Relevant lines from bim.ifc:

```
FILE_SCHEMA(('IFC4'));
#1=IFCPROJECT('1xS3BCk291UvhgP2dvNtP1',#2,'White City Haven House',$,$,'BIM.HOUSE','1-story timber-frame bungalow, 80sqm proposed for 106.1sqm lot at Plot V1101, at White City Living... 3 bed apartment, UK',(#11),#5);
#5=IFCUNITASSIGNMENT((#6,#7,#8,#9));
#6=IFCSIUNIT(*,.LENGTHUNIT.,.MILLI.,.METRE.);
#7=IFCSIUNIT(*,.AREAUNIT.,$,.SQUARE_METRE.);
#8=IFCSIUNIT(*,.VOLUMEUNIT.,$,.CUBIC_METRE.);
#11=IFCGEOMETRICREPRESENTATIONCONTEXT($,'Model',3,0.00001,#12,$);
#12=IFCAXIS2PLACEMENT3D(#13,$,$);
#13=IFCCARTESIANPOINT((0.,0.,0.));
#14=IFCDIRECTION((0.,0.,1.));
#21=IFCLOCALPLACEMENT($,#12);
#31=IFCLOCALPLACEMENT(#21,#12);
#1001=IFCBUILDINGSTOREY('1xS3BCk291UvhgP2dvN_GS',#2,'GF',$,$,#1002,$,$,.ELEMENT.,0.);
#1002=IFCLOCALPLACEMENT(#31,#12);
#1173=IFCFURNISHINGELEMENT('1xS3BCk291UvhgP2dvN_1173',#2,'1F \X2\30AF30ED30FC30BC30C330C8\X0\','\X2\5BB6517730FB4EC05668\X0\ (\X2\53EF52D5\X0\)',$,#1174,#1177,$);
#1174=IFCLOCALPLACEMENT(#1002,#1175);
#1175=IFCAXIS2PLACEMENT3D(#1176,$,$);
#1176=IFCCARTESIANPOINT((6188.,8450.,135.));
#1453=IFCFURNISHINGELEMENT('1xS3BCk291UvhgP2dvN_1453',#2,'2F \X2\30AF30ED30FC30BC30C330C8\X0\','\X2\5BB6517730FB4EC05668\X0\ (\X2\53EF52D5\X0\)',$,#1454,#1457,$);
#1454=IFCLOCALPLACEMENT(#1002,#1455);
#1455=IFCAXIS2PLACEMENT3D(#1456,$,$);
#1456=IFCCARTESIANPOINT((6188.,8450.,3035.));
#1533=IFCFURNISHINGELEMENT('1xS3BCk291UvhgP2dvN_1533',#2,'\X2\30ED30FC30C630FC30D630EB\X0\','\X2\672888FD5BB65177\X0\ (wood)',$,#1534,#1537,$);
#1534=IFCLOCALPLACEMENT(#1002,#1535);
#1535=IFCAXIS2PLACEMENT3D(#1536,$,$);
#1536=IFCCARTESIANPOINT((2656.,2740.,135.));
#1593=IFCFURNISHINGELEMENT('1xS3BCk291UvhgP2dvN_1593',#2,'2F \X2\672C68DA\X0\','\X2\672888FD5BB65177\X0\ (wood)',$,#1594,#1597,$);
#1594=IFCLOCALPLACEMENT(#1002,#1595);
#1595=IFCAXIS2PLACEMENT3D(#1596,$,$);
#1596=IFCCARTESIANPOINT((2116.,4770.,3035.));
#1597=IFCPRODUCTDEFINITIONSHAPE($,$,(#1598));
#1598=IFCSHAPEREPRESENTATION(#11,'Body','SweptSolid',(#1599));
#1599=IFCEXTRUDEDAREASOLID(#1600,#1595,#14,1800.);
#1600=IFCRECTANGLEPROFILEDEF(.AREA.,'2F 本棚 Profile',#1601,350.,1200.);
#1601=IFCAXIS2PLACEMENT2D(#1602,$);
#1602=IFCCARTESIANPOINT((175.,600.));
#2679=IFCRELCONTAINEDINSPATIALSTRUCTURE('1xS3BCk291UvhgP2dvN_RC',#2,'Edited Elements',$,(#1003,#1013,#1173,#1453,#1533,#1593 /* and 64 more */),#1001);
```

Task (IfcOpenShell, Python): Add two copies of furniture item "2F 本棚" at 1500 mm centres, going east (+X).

```python
import numpy as np
import ifcopenshell
import ifcopenshell.api.geometry
import ifcopenshell.api.root
import ifcopenshell.util.element
import ifcopenshell.util.placement
import ifcopenshell.util.unit

model = ifcopenshell.open("bim.ifc")
unit_scale = ifcopenshell.util.unit.calculate_unit_scale(model)


def reuse_history(source, copy):
    """copy_class also copies each property set's owner history, people and application; keep the originals."""
    for rel in copy.IsDefinedBy:
        if rel.is_a("IfcRelDefinesByProperties") and (history := rel.RelatingPropertyDefinition.OwnerHistory):
            rel.RelatingPropertyDefinition.OwnerHistory = source.OwnerHistory
            ifcopenshell.util.element.remove_deep2(model, history)


source = model.by_id(1593)
base = ifcopenshell.util.placement.get_local_placement(source.ObjectPlacement)
step = np.array([1.0, 0.0, 0.0]) * 1.5 / unit_scale

for i in range(1, 3):
    copy = ifcopenshell.api.root.copy_class(model, product=source)
    copy.Representation = ifcopenshell.util.element.copy_deep(
        model, source.Representation, exclude=["IfcGeometricRepresentationContext", "IfcRepresentationMap"]
    )
    reuse_history(source, copy)
    matrix = base.copy()
    matrix[:3, 3] += i * step
    print("added at", matrix[:3, 3].round(3) + 0.0)
    ifcopenshell.api.geometry.edit_object_placement(model, product=copy, matrix=matrix, is_si=False)

model.write("bim_updated.ifc")
```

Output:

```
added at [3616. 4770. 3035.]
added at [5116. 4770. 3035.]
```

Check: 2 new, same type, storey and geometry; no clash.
